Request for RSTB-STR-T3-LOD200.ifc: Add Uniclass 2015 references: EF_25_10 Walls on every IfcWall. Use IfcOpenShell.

First a look at what the model holds.

```python
import ifcopenshell

model = ifcopenshell.open("RSTB-STR-T3-LOD200.ifc")
print(model.schema)
print("classifications:", [c.Name for c in model.by_type("IfcClassification")])
for ifc_class in ("IfcDoor", "IfcRoof", "IfcStair", "IfcWall", "IfcWindow"):
    print(ifc_class, len(model.by_type(ifc_class)))
```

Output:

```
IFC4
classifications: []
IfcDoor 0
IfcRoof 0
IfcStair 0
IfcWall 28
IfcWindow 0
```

```python
import ifcopenshell
import ifcopenshell.api.classification

model = ifcopenshell.open("RSTB-STR-T3-LOD200.ifc")

system = ifcopenshell.api.classification.add_classification(model, classification="Uniclass 2015")

codes = {
    "IfcWall": ("EF_25_10", "Walls"),
}
for ifc_class, (code, name) in codes.items():
    products = model.by_type(ifc_class)
    ifcopenshell.api.classification.add_reference(
        model, products=products, classification=system, identification=code, name=name
    )
    print(code, len(products))

model.write("RSTB-STR-T3-LOD200_edited.ifc")
```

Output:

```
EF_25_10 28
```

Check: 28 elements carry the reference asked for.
